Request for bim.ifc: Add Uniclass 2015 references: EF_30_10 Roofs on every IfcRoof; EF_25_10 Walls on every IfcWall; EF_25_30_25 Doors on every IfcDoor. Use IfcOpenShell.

First a look at what the model holds.

```python
import ifcopenshell

model = ifcopenshell.open("bim.ifc")
print(model.schema)
print("classifications:", [c.Name for c in model.by_type("IfcClassification")])
for ifc_class in ("IfcDoor", "IfcRoof", "IfcStair", "IfcWall", "IfcWindow"):
    print(ifc_class, len(model.by_type(ifc_class)))
```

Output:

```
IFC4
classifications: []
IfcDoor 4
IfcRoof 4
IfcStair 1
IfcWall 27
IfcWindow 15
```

```python
import ifcopenshell
import ifcopenshell.api.classification

model = ifcopenshell.open("bim.ifc")

system = ifcopenshell.api.classification.add_classification(model, classification="Uniclass 2015")

codes = {
    "IfcRoof": ("EF_30_10", "Roofs"),
    "IfcWall": ("EF_25_10", "Walls"),
    "IfcDoor": ("EF_25_30_25", "Doors"),
}
for ifc_class, (code, name) in codes.items():
    products = model.by_type(ifc_class)
    ifcopenshell.api.classification.add_reference(
        model, products=products, classification=system, identification=code, name=name
    )
    print(code, len(products))

model.write("bim_rev.ifc")
```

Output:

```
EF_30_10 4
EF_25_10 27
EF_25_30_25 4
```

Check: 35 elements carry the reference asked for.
